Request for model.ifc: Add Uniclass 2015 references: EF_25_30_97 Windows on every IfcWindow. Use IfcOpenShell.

First a look at what the model holds.

```python
import ifcopenshell

model = ifcopenshell.open("model.ifc")
print(model.schema)
print("classifications:", [c.Name for c in model.by_type("IfcClassification")])
for ifc_class in ("IfcDoor", "IfcRoof", "IfcStair", "IfcWall", "IfcWindow"):
    print(ifc_class, len(model.by_type(ifc_class)))
```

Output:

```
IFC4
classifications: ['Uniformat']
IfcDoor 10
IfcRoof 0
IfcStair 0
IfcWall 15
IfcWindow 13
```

```python
import ifcopenshell
import ifcopenshell.api.classification

model = ifcopenshell.open("model.ifc")

system = ifcopenshell.api.classification.add_classification(model, classification="Uniclass 2015")

codes = {
    "IfcWindow": ("EF_25_30_97", "Windows"),
}
for ifc_class, (code, name) in codes.items():
    products = model.by_type(ifc_class)
    ifcopenshell.api.classification.add_reference(
        model, products=products, classification=system, identification=code, name=name
    )
    print(code, len(products))

model.write("model-out.ifc")
```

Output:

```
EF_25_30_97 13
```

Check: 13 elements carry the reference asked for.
